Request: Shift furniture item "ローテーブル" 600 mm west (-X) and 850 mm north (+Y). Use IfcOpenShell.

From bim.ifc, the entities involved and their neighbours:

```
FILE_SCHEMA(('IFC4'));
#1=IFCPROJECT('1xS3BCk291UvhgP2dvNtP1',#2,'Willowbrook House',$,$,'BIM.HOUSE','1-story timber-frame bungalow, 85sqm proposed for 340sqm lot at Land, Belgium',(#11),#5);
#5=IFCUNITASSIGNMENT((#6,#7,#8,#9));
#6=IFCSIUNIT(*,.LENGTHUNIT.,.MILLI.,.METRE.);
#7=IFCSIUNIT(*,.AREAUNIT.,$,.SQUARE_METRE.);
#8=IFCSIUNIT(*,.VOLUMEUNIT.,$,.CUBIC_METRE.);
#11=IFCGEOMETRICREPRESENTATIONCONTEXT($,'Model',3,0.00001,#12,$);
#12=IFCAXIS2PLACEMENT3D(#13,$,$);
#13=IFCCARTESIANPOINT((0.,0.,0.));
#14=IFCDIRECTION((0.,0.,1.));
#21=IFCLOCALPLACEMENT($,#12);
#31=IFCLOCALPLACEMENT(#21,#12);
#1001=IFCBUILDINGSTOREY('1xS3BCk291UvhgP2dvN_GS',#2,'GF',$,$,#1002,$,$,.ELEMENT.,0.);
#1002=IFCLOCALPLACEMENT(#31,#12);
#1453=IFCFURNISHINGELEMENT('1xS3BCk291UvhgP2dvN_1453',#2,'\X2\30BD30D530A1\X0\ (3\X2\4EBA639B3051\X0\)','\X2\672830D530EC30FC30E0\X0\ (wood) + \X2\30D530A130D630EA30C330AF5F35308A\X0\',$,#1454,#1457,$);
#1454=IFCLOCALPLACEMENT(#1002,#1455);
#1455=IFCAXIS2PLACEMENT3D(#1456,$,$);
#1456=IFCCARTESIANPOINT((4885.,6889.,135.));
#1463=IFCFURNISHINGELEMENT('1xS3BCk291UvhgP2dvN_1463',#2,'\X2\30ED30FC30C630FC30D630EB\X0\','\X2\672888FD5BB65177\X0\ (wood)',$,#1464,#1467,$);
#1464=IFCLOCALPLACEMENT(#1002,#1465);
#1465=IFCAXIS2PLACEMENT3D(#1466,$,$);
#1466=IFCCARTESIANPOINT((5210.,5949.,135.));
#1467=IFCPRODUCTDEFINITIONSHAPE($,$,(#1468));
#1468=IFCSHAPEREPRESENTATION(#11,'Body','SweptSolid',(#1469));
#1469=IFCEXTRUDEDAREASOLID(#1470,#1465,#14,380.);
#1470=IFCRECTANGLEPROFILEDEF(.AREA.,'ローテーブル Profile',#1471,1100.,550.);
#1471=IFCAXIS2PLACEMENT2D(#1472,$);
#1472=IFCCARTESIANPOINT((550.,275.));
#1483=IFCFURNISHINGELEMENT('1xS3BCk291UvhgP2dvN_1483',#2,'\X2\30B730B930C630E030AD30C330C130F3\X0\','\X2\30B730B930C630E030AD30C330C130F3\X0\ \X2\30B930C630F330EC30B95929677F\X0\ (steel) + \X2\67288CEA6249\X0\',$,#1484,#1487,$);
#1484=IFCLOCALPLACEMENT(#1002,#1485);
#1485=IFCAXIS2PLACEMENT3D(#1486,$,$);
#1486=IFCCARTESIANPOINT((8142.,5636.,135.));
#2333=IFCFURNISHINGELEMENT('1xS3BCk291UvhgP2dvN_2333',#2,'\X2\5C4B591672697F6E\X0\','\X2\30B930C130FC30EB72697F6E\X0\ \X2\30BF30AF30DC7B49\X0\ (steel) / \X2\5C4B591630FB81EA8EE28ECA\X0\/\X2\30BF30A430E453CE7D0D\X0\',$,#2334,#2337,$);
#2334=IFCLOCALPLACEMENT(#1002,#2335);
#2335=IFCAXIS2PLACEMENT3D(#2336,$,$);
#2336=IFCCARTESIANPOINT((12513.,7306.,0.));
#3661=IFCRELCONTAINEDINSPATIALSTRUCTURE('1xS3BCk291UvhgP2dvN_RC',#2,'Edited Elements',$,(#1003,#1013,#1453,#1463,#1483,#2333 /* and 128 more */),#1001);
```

```python
import ifcopenshell
import ifcopenshell.api.geometry
import ifcopenshell.util.placement
import ifcopenshell.util.unit

model = ifcopenshell.open("bim.ifc")
unit_scale = ifcopenshell.util.unit.calculate_unit_scale(model)

item = model.by_guid("1xS3BCk291UvhgP2dvN_1463")
matrix = ifcopenshell.util.placement.get_local_placement(item.ObjectPlacement)
matrix[0, 3] -= 0.6 / unit_scale
matrix[1, 3] += 0.85 / unit_scale
ifcopenshell.api.geometry.edit_object_placement(model, product=item, matrix=matrix, is_si=False)

print(ifcopenshell.util.placement.get_local_placement(item.ObjectPlacement).round(3) + 0.0)

model.write("bim-out.ifc")
```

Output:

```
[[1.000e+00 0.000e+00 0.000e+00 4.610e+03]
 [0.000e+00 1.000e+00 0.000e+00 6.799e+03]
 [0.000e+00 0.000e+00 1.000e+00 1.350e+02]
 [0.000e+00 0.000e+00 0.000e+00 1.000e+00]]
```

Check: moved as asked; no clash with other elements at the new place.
